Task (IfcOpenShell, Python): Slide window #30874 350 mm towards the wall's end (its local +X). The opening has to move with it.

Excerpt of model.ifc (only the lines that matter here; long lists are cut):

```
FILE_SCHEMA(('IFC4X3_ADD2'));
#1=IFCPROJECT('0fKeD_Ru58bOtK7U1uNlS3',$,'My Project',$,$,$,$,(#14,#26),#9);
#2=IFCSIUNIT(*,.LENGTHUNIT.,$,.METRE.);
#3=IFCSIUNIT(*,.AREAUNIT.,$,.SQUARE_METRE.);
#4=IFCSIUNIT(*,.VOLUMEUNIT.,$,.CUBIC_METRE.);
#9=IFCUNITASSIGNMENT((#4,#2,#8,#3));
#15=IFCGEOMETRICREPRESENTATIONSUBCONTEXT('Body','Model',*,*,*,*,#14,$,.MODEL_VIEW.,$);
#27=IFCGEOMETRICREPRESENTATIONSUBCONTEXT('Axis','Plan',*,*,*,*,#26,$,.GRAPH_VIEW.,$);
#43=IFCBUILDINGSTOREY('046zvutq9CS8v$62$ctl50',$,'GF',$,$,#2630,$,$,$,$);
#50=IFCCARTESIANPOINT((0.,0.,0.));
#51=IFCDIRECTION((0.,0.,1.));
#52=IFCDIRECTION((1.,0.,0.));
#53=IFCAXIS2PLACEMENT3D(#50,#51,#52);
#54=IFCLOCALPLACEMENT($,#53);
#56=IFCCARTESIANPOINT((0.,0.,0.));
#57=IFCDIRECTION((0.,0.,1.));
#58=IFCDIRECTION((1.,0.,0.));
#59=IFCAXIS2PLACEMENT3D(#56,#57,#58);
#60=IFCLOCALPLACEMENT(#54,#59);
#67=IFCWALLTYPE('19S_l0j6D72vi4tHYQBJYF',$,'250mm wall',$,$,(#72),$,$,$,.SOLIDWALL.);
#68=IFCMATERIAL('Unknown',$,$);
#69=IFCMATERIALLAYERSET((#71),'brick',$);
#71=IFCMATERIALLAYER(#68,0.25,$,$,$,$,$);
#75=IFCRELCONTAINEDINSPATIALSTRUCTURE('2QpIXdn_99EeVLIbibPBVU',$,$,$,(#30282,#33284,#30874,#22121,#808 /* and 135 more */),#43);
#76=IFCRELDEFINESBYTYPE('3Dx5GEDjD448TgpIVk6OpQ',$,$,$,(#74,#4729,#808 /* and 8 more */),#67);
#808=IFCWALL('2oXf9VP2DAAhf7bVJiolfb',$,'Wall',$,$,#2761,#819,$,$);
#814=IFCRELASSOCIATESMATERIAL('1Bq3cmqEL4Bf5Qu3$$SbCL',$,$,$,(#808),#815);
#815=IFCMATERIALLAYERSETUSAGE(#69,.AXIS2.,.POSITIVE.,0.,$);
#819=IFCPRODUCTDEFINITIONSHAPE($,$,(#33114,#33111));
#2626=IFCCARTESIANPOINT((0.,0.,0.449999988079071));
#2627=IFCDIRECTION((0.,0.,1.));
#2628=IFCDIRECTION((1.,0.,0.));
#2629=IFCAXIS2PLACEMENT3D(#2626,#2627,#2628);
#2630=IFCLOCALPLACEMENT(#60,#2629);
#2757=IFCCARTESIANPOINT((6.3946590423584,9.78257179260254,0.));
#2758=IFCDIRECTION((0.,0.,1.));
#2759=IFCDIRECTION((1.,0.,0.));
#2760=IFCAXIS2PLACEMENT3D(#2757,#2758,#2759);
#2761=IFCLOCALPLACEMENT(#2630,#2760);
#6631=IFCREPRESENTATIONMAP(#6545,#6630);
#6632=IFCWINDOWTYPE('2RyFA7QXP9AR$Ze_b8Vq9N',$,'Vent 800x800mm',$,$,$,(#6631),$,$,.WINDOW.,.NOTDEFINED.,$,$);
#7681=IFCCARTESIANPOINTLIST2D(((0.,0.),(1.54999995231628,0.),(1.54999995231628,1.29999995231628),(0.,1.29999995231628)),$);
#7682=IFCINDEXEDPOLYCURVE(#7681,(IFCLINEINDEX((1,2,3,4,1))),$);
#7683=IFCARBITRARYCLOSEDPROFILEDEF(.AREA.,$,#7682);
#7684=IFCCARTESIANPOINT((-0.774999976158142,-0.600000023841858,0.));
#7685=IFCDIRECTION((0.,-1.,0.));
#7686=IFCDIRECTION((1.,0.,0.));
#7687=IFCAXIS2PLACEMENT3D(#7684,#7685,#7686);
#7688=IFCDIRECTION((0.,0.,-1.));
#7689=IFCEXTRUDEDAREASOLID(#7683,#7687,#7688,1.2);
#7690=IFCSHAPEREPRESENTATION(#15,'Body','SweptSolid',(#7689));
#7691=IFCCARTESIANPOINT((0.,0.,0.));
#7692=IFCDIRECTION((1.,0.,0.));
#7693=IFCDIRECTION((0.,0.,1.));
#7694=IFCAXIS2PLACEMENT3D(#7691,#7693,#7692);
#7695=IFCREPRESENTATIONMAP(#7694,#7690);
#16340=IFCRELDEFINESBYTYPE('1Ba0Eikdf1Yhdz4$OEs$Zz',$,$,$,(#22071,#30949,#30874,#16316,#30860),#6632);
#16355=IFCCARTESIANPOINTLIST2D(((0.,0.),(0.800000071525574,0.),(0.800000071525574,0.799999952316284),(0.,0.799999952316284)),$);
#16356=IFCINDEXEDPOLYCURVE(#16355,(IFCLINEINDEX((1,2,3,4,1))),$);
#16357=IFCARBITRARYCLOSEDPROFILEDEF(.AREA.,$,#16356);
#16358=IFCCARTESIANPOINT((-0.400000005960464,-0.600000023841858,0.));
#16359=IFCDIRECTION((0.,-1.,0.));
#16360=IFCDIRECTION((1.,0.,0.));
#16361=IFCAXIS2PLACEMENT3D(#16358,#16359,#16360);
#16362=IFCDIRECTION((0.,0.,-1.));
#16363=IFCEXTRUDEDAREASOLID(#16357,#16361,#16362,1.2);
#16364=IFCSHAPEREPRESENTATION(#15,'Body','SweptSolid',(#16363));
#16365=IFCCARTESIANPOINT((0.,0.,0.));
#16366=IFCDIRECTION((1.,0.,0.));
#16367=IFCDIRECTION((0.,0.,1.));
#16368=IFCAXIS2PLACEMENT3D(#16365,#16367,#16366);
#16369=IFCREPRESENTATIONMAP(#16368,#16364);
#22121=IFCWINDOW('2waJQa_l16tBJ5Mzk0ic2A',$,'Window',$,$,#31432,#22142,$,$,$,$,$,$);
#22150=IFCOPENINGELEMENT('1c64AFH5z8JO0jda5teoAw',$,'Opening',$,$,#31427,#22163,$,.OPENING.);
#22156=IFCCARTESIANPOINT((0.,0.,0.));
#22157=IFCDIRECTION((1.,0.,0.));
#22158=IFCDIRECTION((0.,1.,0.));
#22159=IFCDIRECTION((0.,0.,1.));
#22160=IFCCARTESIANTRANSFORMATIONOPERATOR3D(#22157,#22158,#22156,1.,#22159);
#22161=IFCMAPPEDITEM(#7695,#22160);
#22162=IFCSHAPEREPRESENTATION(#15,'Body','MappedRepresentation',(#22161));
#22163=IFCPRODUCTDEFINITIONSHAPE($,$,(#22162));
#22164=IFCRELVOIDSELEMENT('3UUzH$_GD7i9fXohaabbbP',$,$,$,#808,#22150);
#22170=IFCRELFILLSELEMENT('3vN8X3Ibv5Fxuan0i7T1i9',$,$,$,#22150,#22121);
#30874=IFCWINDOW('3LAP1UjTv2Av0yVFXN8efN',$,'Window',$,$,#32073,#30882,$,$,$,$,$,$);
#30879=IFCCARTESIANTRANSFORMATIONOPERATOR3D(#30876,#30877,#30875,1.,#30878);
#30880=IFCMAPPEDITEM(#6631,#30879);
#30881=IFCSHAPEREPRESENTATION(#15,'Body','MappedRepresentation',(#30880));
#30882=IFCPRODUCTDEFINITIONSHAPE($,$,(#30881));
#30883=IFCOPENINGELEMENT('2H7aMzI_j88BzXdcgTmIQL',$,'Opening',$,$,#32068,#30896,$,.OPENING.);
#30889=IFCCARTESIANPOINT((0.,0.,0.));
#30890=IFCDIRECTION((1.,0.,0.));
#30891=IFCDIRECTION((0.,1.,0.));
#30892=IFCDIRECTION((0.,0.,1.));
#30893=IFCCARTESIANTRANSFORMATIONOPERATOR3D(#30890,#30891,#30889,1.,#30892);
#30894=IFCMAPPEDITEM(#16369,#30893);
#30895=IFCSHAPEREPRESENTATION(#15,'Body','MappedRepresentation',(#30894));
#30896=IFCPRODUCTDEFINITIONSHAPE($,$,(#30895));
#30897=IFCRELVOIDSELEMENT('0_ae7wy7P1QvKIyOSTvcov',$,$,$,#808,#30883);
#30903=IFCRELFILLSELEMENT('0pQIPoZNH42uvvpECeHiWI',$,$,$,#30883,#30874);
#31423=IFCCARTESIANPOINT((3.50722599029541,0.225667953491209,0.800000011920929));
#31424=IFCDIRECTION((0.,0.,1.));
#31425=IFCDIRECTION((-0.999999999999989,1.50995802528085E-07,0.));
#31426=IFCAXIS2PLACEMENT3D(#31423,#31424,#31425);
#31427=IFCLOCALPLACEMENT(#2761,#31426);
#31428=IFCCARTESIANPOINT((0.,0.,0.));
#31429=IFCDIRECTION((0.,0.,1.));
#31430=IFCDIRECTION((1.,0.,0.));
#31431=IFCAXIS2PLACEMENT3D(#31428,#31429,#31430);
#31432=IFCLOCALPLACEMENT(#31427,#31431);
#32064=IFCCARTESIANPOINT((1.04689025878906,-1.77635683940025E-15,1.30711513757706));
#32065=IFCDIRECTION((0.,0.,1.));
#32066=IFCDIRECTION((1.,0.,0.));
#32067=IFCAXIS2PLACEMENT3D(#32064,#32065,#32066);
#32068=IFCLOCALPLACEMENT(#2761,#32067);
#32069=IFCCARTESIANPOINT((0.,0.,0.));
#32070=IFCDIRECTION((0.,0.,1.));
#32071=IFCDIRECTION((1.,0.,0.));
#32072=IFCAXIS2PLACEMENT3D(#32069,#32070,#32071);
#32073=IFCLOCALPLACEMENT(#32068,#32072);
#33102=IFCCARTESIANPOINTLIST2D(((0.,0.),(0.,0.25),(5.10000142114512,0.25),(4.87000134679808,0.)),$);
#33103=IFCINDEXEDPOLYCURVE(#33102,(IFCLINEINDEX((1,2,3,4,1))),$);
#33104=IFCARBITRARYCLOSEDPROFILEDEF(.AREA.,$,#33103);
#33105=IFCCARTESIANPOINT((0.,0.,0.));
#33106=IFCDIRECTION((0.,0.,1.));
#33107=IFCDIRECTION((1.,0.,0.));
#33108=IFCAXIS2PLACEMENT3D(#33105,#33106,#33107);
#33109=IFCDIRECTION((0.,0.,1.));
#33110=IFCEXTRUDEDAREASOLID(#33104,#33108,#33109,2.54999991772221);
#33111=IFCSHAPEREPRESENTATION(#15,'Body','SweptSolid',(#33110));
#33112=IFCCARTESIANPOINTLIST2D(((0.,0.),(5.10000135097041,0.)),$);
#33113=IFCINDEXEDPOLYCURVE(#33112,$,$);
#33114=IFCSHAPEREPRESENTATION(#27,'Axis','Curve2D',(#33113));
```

```python
import ifcopenshell
import ifcopenshell.api.geometry
import ifcopenshell.util.placement
import ifcopenshell.util.unit

model = ifcopenshell.open("model.ifc")
unit_scale = ifcopenshell.util.unit.calculate_unit_scale(model)

window = model.by_guid("3LAP1UjTv2Av0yVFXN8efN")
opening = window.FillsVoids[0].RelatingOpeningElement
wall = opening.VoidsElements[0].RelatingBuildingElement

wall_matrix = ifcopenshell.util.placement.get_local_placement(wall.ObjectPlacement)
shift = wall_matrix[:3, 0] * 0.35 / unit_scale
before = ifcopenshell.util.placement.get_local_placement(window.ObjectPlacement)[:3, 3].copy()

# The window is placed relative to its opening, so it follows when the opening moves.
matrix = ifcopenshell.util.placement.get_local_placement(opening.ObjectPlacement)
matrix[:3, 3] += shift
ifcopenshell.api.geometry.edit_object_placement(
    model, product=opening, matrix=matrix, is_si=False, should_transform_children=True
)

after = ifcopenshell.util.placement.get_local_placement(window.ObjectPlacement)[:3, 3]
print("window moved by", (after - before).round(3) + 0.0)

model.write("model_edited.ifc")
```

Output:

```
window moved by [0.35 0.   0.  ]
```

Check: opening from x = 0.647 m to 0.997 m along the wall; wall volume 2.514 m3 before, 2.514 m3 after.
